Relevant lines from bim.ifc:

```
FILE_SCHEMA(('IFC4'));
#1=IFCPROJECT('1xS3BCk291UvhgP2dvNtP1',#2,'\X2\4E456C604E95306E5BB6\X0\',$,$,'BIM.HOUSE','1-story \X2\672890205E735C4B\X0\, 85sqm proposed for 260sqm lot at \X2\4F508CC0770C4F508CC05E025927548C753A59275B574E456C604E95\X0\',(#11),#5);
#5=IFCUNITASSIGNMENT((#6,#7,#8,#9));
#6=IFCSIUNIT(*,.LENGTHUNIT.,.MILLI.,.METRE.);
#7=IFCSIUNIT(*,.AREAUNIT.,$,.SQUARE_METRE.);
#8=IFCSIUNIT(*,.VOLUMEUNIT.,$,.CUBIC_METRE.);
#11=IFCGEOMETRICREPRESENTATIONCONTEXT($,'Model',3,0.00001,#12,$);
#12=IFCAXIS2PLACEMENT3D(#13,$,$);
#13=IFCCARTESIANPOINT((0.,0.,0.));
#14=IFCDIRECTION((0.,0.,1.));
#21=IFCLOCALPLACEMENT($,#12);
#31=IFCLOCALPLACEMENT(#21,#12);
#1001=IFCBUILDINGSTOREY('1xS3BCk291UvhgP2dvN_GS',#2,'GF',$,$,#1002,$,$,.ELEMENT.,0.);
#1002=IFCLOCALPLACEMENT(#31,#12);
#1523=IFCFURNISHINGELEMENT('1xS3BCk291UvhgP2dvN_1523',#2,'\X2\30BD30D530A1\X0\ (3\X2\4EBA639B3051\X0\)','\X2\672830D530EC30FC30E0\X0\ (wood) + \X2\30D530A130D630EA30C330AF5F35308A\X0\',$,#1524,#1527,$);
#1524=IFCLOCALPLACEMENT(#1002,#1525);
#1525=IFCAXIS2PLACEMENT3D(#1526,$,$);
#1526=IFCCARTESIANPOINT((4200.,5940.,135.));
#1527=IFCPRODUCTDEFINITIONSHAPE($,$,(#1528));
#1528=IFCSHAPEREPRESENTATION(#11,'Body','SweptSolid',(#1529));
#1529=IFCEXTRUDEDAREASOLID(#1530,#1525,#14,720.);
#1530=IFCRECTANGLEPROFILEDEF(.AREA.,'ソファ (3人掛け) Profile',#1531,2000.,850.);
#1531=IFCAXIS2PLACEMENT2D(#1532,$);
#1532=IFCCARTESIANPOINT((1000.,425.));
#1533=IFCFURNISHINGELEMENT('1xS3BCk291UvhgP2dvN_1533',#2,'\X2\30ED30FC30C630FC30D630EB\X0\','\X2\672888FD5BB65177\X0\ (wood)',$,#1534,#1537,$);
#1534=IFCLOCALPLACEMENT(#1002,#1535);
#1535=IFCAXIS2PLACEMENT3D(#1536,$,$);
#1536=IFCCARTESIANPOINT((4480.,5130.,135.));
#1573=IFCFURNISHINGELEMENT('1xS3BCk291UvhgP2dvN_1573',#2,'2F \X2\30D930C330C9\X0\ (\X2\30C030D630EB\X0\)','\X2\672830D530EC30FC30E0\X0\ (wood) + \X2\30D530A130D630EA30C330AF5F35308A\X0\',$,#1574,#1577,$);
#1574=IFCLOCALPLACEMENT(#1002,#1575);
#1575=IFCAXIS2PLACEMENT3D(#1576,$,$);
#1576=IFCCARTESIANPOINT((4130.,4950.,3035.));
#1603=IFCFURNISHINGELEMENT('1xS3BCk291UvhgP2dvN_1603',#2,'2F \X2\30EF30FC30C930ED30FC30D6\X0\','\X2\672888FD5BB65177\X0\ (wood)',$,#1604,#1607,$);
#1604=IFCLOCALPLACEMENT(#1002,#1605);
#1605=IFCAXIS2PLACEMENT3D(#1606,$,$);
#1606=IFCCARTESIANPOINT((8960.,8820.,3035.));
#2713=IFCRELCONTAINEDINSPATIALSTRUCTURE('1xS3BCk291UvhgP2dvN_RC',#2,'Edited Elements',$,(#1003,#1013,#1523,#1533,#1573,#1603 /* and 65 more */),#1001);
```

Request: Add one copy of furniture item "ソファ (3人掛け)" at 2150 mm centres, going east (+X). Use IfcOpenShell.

```python
import numpy as np
import ifcopenshell
import ifcopenshell.api.geometry
import ifcopenshell.api.root
import ifcopenshell.util.element
import ifcopenshell.util.placement
import ifcopenshell.util.unit

model = ifcopenshell.open("bim.ifc")
unit_scale = ifcopenshell.util.unit.calculate_unit_scale(model)


def reuse_history(source, copy):
    """copy_class also copies each property set's owner history, people and application; keep the originals."""
    for rel in copy.IsDefinedBy:
        if rel.is_a("IfcRelDefinesByProperties") and (history := rel.RelatingPropertyDefinition.OwnerHistory):
            rel.RelatingPropertyDefinition.OwnerHistory = source.OwnerHistory
            ifcopenshell.util.element.remove_deep2(model, history)


source = model.by_id(1523)
base = ifcopenshell.util.placement.get_local_placement(source.ObjectPlacement)
step = np.array([1.0, 0.0, 0.0]) * 2.15 / unit_scale

for i in range(1, 2):
    copy = ifcopenshell.api.root.copy_class(model, product=source)
    copy.Representation = ifcopenshell.util.element.copy_deep(
        model, source.Representation, exclude=["IfcGeometricRepresentationContext", "IfcRepresentationMap"]
    )
    reuse_history(source, copy)
    matrix = base.copy()
    matrix[:3, 3] += i * step
    print("added at", matrix[:3, 3].round(3) + 0.0)
    ifcopenshell.api.geometry.edit_object_placement(model, product=copy, matrix=matrix, is_si=False)

model.write("bim_edited.ifc")
```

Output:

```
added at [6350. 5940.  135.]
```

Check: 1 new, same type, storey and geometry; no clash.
